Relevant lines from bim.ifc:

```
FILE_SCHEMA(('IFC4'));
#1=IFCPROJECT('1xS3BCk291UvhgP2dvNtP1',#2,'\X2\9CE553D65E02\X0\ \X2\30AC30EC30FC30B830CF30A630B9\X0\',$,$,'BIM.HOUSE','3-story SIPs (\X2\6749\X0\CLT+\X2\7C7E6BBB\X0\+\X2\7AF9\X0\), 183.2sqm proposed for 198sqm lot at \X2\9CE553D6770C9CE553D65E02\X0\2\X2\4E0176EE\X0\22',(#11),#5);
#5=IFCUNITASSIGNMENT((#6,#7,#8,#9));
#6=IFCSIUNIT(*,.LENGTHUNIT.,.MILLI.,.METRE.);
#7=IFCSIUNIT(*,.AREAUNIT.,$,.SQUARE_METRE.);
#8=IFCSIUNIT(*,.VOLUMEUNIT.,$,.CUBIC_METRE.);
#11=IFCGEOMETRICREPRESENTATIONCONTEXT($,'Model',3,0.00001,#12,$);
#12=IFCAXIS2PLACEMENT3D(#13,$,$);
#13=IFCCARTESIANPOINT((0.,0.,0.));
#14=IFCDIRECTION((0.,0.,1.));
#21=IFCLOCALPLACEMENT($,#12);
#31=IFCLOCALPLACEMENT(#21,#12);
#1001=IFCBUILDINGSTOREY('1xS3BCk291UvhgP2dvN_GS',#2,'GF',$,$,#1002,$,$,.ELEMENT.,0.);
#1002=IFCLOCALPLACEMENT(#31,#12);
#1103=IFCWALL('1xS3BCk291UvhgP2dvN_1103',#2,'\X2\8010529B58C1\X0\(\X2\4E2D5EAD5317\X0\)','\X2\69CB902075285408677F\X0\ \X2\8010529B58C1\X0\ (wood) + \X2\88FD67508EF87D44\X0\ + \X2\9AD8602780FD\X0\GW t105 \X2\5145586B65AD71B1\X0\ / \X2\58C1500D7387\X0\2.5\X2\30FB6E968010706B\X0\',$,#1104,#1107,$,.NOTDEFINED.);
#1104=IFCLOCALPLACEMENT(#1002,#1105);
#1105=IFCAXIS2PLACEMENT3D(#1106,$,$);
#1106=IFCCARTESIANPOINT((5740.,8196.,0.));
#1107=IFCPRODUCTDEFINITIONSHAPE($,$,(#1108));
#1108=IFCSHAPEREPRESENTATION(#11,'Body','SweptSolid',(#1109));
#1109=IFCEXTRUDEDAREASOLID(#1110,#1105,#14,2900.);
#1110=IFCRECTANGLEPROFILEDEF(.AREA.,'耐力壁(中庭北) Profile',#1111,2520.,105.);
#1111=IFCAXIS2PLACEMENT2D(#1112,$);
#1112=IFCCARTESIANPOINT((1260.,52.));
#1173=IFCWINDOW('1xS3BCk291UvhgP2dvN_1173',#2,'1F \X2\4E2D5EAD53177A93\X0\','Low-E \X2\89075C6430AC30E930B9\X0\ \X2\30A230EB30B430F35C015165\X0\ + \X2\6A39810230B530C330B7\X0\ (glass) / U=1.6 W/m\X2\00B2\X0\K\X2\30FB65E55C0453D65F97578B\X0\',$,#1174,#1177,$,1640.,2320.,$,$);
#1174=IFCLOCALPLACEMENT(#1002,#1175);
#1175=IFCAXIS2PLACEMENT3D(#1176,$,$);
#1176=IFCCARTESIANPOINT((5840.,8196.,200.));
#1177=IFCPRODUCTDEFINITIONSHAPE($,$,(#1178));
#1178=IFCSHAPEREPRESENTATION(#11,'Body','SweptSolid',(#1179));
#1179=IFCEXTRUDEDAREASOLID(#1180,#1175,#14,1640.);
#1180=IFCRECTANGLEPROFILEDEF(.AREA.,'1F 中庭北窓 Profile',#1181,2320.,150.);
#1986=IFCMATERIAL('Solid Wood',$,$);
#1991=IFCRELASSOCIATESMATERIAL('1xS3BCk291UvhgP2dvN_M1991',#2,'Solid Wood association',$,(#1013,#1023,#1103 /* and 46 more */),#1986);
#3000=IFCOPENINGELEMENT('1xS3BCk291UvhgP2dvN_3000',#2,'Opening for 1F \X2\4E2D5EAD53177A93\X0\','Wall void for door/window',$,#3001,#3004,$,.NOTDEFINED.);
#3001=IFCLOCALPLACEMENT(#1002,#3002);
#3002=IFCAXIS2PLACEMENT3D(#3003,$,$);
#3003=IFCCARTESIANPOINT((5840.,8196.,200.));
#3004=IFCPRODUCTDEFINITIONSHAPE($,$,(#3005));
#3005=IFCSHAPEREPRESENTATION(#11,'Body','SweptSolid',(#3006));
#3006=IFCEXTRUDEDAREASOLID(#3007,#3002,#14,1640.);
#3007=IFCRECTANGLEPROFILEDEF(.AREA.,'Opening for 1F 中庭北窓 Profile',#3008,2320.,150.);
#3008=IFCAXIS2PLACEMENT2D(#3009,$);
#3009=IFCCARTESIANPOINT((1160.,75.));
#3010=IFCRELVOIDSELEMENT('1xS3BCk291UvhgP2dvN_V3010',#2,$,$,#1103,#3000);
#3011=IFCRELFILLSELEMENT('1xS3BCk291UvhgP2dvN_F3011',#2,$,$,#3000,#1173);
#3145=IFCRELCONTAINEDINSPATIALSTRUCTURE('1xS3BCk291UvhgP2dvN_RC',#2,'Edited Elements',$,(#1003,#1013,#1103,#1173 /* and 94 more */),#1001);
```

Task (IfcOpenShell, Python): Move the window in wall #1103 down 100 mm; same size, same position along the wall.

```python
import numpy as np
import ifcopenshell
import ifcopenshell.api.geometry
import ifcopenshell.util.placement
import ifcopenshell.util.unit

model = ifcopenshell.open("bim.ifc")
unit_scale = ifcopenshell.util.unit.calculate_unit_scale(model)

window = model.by_guid("1xS3BCk291UvhgP2dvN_1173")
opening = window.FillsVoids[0].RelatingOpeningElement
dz = -0.1 / unit_scale

shift = np.array([0.0, 0.0, dz])
# The window is not placed relative to its opening, so move both.
for product in (opening, window):
    matrix = ifcopenshell.util.placement.get_local_placement(product.ObjectPlacement)
    matrix[:3, 3] += shift
    ifcopenshell.api.geometry.edit_object_placement(model, product=product, matrix=matrix, is_si=False)

print(f"moved by {dz * unit_scale:+.3f} m")

model.write("bim_updated.ifc")
```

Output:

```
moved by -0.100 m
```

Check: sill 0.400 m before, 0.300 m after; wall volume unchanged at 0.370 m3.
